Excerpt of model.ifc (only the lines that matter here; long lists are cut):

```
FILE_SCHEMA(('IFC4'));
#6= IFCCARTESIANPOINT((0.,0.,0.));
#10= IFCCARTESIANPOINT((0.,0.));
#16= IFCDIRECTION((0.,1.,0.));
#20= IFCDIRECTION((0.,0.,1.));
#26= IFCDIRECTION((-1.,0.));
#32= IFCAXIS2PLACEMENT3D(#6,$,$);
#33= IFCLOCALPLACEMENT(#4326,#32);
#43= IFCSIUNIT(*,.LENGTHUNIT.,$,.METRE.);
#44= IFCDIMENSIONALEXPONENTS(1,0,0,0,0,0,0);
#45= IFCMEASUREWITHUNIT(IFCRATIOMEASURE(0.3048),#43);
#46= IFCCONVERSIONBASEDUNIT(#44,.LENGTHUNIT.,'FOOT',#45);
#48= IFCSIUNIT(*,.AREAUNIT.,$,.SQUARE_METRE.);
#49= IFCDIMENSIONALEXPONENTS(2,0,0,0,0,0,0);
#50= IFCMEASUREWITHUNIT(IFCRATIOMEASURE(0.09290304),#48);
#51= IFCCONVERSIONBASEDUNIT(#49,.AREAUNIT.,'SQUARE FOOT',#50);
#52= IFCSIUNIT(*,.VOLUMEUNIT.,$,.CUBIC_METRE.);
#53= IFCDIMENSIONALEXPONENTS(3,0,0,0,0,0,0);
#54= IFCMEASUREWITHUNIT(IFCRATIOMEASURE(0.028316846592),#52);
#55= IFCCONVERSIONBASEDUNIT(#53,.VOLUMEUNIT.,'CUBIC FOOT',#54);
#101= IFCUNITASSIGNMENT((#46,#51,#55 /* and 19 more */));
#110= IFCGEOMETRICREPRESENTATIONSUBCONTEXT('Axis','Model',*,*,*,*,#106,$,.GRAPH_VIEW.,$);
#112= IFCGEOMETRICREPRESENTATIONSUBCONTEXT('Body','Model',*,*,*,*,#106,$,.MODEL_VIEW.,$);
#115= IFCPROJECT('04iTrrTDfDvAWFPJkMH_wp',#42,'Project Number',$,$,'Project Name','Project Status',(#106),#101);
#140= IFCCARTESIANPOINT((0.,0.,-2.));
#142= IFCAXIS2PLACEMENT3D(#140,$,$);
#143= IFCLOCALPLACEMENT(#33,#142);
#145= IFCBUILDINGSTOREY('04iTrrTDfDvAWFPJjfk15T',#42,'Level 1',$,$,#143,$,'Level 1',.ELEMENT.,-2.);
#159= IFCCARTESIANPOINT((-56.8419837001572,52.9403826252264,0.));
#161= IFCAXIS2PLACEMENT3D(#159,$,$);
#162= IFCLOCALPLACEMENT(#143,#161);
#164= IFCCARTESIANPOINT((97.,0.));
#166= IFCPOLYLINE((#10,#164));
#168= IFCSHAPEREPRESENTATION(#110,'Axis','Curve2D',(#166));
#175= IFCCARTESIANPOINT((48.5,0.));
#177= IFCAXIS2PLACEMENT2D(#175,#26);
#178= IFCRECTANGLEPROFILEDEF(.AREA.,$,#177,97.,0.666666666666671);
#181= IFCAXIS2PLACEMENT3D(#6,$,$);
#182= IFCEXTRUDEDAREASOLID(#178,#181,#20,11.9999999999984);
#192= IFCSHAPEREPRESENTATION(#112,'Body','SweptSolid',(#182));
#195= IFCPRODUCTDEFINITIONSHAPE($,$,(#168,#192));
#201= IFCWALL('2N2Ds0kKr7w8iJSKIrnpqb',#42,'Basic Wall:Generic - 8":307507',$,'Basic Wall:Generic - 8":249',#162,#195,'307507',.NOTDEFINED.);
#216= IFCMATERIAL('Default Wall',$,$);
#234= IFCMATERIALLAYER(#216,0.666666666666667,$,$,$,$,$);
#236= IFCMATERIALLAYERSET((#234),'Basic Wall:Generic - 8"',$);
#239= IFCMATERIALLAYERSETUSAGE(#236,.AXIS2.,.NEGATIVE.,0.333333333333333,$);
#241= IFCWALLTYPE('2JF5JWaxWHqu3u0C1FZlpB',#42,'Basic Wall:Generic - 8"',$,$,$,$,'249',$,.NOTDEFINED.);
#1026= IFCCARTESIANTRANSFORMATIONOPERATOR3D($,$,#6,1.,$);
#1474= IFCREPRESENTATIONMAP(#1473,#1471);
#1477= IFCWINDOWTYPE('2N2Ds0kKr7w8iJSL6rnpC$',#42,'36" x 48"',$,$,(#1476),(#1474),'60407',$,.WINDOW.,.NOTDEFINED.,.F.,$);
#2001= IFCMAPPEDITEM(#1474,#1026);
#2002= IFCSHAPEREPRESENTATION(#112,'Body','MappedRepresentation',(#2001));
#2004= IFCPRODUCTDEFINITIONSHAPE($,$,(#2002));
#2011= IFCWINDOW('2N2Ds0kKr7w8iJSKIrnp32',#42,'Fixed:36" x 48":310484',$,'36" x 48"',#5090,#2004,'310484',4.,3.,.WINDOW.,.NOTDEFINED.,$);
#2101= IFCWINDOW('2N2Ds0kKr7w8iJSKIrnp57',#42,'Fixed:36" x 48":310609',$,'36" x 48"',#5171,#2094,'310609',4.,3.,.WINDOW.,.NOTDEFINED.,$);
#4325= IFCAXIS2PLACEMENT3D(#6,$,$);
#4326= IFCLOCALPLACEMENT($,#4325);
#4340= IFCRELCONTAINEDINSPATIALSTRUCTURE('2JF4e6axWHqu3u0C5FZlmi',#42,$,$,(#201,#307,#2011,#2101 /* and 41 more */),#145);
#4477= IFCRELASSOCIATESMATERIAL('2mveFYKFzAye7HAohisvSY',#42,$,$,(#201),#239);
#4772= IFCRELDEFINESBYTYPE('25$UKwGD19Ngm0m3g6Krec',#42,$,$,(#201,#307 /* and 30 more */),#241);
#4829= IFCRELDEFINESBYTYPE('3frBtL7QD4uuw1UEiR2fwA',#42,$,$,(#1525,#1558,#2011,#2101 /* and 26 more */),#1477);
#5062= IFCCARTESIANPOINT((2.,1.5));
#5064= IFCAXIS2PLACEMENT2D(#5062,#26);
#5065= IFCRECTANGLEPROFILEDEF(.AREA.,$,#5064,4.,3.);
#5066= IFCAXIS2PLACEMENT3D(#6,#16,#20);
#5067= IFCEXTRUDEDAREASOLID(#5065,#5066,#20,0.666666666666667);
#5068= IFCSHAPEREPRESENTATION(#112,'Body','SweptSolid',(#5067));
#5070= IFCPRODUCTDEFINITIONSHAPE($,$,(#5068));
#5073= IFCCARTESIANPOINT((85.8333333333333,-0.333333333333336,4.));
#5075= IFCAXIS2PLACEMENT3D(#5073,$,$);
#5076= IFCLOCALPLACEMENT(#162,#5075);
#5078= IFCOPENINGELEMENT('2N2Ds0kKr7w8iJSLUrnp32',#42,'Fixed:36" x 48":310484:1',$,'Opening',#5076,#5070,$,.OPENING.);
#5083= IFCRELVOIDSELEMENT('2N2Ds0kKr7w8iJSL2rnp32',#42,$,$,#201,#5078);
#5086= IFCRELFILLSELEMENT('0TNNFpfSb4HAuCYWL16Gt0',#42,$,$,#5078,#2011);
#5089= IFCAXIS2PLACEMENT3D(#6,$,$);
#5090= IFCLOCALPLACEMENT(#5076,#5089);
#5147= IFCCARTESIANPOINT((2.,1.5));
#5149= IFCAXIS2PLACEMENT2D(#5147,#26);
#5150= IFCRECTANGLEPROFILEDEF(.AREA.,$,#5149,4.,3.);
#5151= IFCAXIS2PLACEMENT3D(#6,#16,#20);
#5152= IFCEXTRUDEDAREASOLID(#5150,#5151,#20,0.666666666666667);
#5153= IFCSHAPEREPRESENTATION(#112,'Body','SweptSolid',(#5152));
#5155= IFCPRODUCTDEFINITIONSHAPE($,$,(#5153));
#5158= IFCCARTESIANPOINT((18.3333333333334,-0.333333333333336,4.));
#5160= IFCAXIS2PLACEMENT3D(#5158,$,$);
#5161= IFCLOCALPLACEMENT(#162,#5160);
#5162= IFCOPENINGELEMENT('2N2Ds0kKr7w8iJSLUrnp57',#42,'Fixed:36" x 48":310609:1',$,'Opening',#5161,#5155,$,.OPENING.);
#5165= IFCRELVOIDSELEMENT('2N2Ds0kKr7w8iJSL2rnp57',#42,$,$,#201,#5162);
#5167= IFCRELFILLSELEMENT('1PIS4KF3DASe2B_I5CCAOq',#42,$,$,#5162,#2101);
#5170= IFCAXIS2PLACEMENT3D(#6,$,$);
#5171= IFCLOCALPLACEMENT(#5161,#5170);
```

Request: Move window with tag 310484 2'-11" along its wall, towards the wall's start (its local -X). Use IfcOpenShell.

```python
import ifcopenshell
import ifcopenshell.api.geometry
import ifcopenshell.util.placement
import ifcopenshell.util.unit

model = ifcopenshell.open("model.ifc")
unit_scale = ifcopenshell.util.unit.calculate_unit_scale(model)

window = model.by_id(2011)
opening = window.FillsVoids[0].RelatingOpeningElement
wall = opening.VoidsElements[0].RelatingBuildingElement

wall_matrix = ifcopenshell.util.placement.get_local_placement(wall.ObjectPlacement)
shift = wall_matrix[:3, 0] * -35 * 0.0254 / unit_scale
before = ifcopenshell.util.placement.get_local_placement(window.ObjectPlacement)[:3, 3].copy()

# The window is placed relative to its opening, so it follows when the opening moves.
matrix = ifcopenshell.util.placement.get_local_placement(opening.ObjectPlacement)
matrix[:3, 3] += shift
ifcopenshell.api.geometry.edit_object_placement(
    model, product=opening, matrix=matrix, is_si=False, should_transform_children=True
)

after = ifcopenshell.util.placement.get_local_placement(window.ObjectPlacement)[:3, 3]
print("window moved by", (after - before).round(3) + 0.0)

model.write("model_rev.ifc")
```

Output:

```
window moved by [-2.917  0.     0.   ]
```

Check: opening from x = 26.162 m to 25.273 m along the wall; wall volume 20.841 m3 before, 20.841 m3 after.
